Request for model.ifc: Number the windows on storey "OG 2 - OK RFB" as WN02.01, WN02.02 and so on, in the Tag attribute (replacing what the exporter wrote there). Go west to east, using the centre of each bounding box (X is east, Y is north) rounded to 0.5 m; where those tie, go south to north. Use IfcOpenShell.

First a look at what the model holds.

```python
import ifcopenshell
import ifcopenshell.util.element
import ifcopenshell.util.placement

model = ifcopenshell.open("model.ifc")
print(model.schema)
storey = next(s for s in model.by_type("IfcBuildingStorey") if s.Name == "OG 2 - OK RFB")
windows = [e for e in ifcopenshell.util.element.get_decomposition(storey) if e.is_a("IfcWindow")]
for e in sorted(windows, key=lambda e: e.id()):
    origin = ifcopenshell.util.placement.get_local_placement(e.ObjectPlacement)[:3, 3]
    print(e.id(), e.Tag, e.Name, origin.round(2) + 0.0, sep=" | ")
```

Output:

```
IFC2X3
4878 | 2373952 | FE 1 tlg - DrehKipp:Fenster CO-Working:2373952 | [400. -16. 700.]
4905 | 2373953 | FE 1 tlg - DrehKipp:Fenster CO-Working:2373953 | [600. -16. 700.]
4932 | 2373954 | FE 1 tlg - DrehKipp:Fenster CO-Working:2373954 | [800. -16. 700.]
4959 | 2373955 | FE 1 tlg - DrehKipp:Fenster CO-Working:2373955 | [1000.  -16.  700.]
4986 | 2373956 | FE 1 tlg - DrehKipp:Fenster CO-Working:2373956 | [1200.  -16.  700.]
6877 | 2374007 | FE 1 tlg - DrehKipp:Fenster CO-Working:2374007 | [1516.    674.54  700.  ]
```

```python
import ifcopenshell
import ifcopenshell.geom
import ifcopenshell.util.element
import ifcopenshell.util.shape

model = ifcopenshell.open("model.ifc")
settings = ifcopenshell.geom.settings()
settings.set("use-world-coords", True)


def centre(element):
    shape = ifcopenshell.geom.create_shape(settings, element)
    return ifcopenshell.util.shape.get_bbox_centroid(shape.geometry)


storey = next(s for s in model.by_type("IfcBuildingStorey") if s.Name == "OG 2 - OK RFB")
windows = [e for e in ifcopenshell.util.element.get_decomposition(storey) if e.is_a("IfcWindow")]

# Insertion points can sit at a corner or the storey origin, so sort by the geometry (in metres).
centres = {e: centre(e) for e in windows}
windows.sort(key=lambda e: (round(centres[e][0] / 0.5), centres[e][1]))

for i, e in enumerate(windows, start=1):
    number = f"WN02.{i:02d}"
    e.Tag = number
    print(e.id(), number)

model.write("model_rev.ifc")
```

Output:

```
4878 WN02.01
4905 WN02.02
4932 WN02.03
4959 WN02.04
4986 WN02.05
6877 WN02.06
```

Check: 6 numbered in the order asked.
